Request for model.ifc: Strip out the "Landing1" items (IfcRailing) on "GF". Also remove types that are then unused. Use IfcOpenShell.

First a look at what the model holds.

```python
import ifcopenshell
import ifcopenshell.util.element

model = ifcopenshell.open("model.ifc")
print(model.schema)
storey = next(s for s in model.by_type("IfcBuildingStorey") if s.Name == "GF")
railings = [e for e in ifcopenshell.util.element.get_decomposition(storey) if e.is_a("IfcRailing")]
seen = {}
for e in railings:
    element_type = ifcopenshell.util.element.get_type(e)
    name = element_type.Name if element_type not in (None, e) else None
    seen[name] = seen.get(name, 0) + 1
for name, count in sorted(seen.items(), key=str):
    print(count, "x", name)
```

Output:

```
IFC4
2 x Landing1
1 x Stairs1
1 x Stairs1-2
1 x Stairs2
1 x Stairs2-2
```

```python
import ifcopenshell
import ifcopenshell.api.root
import ifcopenshell.util.element

model = ifcopenshell.open("model.ifc")

storey = next(s for s in model.by_type("IfcBuildingStorey") if s.Name == "GF")
railings = [e for e in ifcopenshell.util.element.get_decomposition(storey) if e.is_a("IfcRailing")]
targets = [e for e in railings if (t := ifcopenshell.util.element.get_type(e)) not in (None, e) and t.Name == "Landing1"]
types = {ifcopenshell.util.element.get_type(e) for e in targets} - {None, *targets}

for e in targets:
    ifcopenshell.api.root.remove_product(model, product=e)
print(len(targets), "removed")

unused = [t for t in types if not ifcopenshell.util.element.get_types(t)]
for t in unused:
    ifcopenshell.api.root.remove_product(model, product=t)
print(len(unused), "unused types removed")

model.write("model-out.ifc")
```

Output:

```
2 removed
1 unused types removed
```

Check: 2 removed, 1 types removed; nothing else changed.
